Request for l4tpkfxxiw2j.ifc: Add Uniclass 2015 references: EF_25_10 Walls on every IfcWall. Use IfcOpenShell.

First a look at what the model holds.

```python
import ifcopenshell

model = ifcopenshell.open("l4tpkfxxiw2j.ifc")
print(model.schema)
print("classifications:", [c.Name for c in model.by_type("IfcClassification")])
for ifc_class in ("IfcDoor", "IfcRoof", "IfcStair", "IfcWall", "IfcWindow"):
    print(ifc_class, len(model.by_type(ifc_class)))
```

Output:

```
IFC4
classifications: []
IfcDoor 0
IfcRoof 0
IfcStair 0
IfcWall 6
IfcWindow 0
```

```python
import ifcopenshell
import ifcopenshell.api.classification

model = ifcopenshell.open("l4tpkfxxiw2j.ifc")

system = ifcopenshell.api.classification.add_classification(model, classification="Uniclass 2015")

codes = {
    "IfcWall": ("EF_25_10", "Walls"),
}
for ifc_class, (code, name) in codes.items():
    products = model.by_type(ifc_class)
    ifcopenshell.api.classification.add_reference(
        model, products=products, classification=system, identification=code, name=name
    )
    print(code, len(products))

model.write("l4tpkfxxiw2j-out.ifc")
```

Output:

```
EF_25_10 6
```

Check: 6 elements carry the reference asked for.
